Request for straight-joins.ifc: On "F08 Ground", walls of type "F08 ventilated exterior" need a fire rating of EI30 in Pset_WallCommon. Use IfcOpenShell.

First a look at what the model holds.

```python
import ifcopenshell
import ifcopenshell.util.element

model = ifcopenshell.open("straight-joins.ifc")
print(model.schema)
storey = next(s for s in model.by_type("IfcBuildingStorey") if s.Name == "F08 Ground")
walls = [e for e in ifcopenshell.util.element.get_decomposition(storey) if e.is_a("IfcWall")]
seen = {}
for e in walls:
    element_type = ifcopenshell.util.element.get_type(e)
    key = (element_type.Name if element_type != e and element_type else None, ifcopenshell.util.element.get_pset(e, "Pset_WallCommon", "FireRating"))
    seen[key] = seen.get(key, 0) + 1
for (name, value), count in sorted(seen.items(), key=str):
    print(count, "x", name, "|", value)
```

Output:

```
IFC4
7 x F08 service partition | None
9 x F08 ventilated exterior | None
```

```python
import ifcopenshell
import ifcopenshell.api.pset
import ifcopenshell.util.element

model = ifcopenshell.open("straight-joins.ifc")

storey = next(s for s in model.by_type("IfcBuildingStorey") if s.Name == "F08 Ground")
walls = [e for e in ifcopenshell.util.element.get_decomposition(storey) if e.is_a("IfcWall")]

count = 0
for e in walls:
    element_type = ifcopenshell.util.element.get_type(e)
    if element_type in (None, e) or element_type.Name != "F08 ventilated exterior":
        continue
    # add_pset returns the element's existing set when there is one.
    pset = ifcopenshell.api.pset.add_pset(model, product=e, name="Pset_WallCommon")
    ifcopenshell.api.pset.edit_pset(model, pset=pset, properties={"FireRating": "EI30"})
    count += 1

print(count, "walls updated")

model.write("straight-joins_rev.ifc")
```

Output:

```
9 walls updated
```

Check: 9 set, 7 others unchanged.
